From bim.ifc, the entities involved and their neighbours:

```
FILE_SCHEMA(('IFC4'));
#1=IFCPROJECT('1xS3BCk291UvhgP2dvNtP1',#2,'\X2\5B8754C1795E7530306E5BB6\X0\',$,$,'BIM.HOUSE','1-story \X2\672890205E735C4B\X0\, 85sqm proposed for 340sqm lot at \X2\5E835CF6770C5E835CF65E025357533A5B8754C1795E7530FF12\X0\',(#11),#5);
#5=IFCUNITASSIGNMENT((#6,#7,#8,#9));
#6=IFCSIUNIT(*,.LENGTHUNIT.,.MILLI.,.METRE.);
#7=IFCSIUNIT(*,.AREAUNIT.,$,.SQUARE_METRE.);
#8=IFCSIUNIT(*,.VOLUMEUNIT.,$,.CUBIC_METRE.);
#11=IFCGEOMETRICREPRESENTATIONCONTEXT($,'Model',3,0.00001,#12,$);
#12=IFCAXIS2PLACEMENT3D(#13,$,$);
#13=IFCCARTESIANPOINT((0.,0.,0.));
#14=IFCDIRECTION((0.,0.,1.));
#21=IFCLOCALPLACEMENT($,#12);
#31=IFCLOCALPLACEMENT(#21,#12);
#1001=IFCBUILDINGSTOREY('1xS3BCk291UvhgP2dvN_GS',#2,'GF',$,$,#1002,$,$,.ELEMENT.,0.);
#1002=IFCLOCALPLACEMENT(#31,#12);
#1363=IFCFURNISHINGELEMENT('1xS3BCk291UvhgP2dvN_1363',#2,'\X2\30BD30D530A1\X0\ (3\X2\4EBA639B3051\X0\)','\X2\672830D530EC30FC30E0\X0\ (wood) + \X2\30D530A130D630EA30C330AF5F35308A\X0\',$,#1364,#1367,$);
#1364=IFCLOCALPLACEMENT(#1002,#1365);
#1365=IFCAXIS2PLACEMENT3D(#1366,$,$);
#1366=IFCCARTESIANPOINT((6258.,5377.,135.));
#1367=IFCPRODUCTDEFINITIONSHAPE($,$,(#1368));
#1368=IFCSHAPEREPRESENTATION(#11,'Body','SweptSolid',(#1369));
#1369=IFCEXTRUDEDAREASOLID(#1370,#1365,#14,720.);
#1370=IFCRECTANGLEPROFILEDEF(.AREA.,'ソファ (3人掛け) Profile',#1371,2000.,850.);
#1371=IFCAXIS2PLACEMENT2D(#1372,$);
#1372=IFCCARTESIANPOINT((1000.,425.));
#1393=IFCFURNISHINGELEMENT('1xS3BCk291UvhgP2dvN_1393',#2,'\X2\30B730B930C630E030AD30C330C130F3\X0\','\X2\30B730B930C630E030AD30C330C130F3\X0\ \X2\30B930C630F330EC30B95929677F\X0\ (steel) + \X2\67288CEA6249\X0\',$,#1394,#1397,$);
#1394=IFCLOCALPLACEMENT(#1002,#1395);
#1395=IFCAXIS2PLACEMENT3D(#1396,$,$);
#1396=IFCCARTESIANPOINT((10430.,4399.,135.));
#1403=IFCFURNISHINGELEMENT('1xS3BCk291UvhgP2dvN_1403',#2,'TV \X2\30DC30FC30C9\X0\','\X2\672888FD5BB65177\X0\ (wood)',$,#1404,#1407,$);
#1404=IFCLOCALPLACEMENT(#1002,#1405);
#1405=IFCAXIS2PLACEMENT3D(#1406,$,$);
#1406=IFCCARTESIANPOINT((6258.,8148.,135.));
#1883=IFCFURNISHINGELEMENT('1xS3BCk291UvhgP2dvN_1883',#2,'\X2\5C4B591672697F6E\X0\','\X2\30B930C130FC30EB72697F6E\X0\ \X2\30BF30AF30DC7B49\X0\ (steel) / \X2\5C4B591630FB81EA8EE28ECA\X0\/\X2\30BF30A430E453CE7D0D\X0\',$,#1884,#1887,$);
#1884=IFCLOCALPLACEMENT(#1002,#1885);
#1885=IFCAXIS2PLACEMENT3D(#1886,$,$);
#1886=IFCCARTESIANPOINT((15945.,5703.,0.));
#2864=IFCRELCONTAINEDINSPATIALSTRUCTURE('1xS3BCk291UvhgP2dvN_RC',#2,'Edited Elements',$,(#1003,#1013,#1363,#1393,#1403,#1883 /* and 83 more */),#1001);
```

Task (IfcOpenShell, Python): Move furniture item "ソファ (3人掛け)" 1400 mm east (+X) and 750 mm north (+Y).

```python
import ifcopenshell
import ifcopenshell.api.geometry
import ifcopenshell.util.placement
import ifcopenshell.util.unit

model = ifcopenshell.open("bim.ifc")
unit_scale = ifcopenshell.util.unit.calculate_unit_scale(model)

item = model.by_id(1363)
matrix = ifcopenshell.util.placement.get_local_placement(item.ObjectPlacement)
matrix[0, 3] += 1.4 / unit_scale
matrix[1, 3] += 0.75 / unit_scale
ifcopenshell.api.geometry.edit_object_placement(model, product=item, matrix=matrix, is_si=False)

print(ifcopenshell.util.placement.get_local_placement(item.ObjectPlacement).round(3) + 0.0)

model.write("bim_v2.ifc")
```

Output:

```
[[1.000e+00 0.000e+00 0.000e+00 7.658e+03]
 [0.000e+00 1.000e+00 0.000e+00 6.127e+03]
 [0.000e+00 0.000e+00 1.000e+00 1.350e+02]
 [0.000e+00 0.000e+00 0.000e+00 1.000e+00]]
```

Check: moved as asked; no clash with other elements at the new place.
